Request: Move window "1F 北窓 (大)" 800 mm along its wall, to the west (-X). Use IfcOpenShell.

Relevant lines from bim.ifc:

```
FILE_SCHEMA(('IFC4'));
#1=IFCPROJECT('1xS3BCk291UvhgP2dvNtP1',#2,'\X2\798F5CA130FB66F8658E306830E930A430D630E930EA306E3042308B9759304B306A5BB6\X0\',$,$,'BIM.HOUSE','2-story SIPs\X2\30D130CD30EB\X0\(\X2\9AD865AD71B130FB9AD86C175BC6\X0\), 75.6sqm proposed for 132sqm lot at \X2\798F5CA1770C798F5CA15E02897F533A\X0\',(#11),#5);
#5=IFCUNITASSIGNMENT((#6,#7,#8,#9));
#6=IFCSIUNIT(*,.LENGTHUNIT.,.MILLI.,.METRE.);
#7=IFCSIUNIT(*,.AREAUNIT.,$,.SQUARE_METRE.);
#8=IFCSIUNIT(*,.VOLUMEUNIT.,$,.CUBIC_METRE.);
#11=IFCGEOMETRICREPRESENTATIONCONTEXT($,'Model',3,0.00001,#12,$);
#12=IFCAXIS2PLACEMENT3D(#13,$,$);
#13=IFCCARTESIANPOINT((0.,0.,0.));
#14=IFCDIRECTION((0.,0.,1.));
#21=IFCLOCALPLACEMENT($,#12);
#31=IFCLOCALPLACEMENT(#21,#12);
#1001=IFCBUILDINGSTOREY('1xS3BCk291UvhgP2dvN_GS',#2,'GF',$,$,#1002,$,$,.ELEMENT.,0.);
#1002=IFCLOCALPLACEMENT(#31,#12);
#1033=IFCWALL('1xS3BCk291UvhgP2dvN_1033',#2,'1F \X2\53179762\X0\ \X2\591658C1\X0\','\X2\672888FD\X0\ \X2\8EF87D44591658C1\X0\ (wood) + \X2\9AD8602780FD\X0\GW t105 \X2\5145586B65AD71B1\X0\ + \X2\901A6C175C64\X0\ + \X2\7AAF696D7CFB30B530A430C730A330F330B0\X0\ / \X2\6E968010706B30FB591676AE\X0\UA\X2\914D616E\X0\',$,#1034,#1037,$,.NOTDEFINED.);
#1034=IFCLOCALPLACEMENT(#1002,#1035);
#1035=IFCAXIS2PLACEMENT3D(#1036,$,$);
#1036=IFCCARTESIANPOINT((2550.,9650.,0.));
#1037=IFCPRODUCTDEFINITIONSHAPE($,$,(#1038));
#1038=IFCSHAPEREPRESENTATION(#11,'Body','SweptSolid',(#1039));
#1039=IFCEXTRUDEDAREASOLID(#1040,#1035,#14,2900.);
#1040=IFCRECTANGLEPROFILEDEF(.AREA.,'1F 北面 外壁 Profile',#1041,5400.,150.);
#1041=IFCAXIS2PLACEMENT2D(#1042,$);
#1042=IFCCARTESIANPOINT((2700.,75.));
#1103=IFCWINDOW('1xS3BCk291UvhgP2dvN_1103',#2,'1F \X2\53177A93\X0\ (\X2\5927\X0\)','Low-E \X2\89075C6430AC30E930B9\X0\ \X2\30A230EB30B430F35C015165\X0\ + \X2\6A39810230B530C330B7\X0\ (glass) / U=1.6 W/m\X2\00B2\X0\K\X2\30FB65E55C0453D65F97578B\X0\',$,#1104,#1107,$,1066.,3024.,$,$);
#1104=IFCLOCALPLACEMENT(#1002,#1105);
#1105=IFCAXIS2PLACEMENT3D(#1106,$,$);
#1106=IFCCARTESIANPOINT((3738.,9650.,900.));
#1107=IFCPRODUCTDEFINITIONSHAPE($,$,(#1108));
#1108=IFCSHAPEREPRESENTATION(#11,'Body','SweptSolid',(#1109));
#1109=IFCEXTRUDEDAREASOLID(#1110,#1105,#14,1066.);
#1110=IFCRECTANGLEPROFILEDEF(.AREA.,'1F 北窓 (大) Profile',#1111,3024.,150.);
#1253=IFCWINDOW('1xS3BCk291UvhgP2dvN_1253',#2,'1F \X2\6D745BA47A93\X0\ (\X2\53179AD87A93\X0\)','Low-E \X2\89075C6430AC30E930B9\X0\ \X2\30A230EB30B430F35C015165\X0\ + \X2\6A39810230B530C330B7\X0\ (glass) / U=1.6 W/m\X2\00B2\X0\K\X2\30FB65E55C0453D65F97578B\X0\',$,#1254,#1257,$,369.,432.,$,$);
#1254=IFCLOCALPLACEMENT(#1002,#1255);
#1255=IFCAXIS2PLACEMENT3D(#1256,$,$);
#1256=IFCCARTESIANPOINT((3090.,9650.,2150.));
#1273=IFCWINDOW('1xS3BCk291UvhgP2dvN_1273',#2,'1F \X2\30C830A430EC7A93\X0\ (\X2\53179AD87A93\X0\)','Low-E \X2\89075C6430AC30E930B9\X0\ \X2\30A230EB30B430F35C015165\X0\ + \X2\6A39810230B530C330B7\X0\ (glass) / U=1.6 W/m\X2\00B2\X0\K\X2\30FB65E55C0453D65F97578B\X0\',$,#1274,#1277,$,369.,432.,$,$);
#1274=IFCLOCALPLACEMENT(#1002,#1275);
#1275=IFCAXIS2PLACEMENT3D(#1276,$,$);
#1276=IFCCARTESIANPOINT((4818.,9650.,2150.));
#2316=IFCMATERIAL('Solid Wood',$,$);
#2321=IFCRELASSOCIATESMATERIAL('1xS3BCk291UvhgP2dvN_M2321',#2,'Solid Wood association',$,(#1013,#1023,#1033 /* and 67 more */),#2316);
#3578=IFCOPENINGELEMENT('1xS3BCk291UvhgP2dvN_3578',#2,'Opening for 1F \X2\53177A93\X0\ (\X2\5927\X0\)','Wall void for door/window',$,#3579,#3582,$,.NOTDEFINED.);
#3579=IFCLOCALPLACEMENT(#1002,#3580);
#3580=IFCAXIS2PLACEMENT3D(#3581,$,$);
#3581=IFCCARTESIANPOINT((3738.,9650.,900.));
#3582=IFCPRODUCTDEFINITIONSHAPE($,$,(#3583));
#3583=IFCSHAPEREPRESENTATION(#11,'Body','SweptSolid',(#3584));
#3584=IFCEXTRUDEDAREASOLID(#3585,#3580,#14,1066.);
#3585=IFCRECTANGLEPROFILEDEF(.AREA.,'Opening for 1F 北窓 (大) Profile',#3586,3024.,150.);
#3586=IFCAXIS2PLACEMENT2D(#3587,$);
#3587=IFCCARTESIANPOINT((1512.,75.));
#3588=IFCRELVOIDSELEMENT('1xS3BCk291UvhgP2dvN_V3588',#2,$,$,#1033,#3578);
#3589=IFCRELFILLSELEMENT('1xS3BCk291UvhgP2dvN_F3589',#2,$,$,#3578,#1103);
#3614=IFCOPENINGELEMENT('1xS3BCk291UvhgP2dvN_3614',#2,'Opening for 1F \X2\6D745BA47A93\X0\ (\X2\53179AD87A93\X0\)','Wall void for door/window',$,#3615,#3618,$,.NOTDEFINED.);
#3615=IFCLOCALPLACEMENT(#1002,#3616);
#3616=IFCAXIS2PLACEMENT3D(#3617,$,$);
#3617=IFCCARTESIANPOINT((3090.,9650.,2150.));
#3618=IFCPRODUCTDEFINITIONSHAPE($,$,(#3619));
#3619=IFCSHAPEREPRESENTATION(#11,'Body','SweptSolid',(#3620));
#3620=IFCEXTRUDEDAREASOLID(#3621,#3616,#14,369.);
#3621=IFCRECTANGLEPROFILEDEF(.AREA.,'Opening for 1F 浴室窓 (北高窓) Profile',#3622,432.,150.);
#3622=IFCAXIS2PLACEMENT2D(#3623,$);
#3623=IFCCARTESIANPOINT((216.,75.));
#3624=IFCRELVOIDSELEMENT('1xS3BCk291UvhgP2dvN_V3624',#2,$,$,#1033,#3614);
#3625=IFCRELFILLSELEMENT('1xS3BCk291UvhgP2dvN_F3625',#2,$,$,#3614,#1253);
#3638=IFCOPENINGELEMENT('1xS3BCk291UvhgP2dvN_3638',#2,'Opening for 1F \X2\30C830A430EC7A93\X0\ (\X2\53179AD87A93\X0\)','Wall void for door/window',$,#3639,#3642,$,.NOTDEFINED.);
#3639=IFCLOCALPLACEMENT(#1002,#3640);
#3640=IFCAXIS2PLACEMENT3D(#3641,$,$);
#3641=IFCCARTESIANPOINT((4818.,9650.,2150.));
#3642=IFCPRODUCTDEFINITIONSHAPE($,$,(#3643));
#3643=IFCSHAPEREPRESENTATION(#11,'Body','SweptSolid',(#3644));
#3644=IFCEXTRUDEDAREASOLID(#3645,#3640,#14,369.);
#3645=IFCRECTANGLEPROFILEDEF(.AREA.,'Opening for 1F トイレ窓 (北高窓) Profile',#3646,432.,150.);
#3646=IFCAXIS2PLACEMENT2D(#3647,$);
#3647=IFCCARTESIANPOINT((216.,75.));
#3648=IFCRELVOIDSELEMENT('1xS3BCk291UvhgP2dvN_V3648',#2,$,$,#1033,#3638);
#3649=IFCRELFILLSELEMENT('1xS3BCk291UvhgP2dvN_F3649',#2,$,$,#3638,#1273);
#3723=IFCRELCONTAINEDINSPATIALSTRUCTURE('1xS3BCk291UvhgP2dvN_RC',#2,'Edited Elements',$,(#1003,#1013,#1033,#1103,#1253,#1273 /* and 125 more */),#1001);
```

```python
import ifcopenshell
import ifcopenshell.api.geometry
import ifcopenshell.util.placement

model = ifcopenshell.open("bim.ifc")

window = model.by_guid("1xS3BCk291UvhgP2dvN_1103")
opening = window.FillsVoids[0].RelatingOpeningElement
wall = opening.VoidsElements[0].RelatingBuildingElement

wall_matrix = ifcopenshell.util.placement.get_local_placement(wall.ObjectPlacement)
shift = wall_matrix[:3, 0] * -800.0
before = ifcopenshell.util.placement.get_local_placement(window.ObjectPlacement)[:3, 3].copy()

# The window is not placed relative to its opening, so move both.
for product in (opening, window):
    matrix = ifcopenshell.util.placement.get_local_placement(product.ObjectPlacement)
    matrix[:3, 3] += shift
    ifcopenshell.api.geometry.edit_object_placement(model, product=product, matrix=matrix, is_si=False)

after = ifcopenshell.util.placement.get_local_placement(window.ObjectPlacement)[:3, 3]
print("window moved by", (after - before).round(3) + 0.0)

model.write("bim_rev.ifc")
```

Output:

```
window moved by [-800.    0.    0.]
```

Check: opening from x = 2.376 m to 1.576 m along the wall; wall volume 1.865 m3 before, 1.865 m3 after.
